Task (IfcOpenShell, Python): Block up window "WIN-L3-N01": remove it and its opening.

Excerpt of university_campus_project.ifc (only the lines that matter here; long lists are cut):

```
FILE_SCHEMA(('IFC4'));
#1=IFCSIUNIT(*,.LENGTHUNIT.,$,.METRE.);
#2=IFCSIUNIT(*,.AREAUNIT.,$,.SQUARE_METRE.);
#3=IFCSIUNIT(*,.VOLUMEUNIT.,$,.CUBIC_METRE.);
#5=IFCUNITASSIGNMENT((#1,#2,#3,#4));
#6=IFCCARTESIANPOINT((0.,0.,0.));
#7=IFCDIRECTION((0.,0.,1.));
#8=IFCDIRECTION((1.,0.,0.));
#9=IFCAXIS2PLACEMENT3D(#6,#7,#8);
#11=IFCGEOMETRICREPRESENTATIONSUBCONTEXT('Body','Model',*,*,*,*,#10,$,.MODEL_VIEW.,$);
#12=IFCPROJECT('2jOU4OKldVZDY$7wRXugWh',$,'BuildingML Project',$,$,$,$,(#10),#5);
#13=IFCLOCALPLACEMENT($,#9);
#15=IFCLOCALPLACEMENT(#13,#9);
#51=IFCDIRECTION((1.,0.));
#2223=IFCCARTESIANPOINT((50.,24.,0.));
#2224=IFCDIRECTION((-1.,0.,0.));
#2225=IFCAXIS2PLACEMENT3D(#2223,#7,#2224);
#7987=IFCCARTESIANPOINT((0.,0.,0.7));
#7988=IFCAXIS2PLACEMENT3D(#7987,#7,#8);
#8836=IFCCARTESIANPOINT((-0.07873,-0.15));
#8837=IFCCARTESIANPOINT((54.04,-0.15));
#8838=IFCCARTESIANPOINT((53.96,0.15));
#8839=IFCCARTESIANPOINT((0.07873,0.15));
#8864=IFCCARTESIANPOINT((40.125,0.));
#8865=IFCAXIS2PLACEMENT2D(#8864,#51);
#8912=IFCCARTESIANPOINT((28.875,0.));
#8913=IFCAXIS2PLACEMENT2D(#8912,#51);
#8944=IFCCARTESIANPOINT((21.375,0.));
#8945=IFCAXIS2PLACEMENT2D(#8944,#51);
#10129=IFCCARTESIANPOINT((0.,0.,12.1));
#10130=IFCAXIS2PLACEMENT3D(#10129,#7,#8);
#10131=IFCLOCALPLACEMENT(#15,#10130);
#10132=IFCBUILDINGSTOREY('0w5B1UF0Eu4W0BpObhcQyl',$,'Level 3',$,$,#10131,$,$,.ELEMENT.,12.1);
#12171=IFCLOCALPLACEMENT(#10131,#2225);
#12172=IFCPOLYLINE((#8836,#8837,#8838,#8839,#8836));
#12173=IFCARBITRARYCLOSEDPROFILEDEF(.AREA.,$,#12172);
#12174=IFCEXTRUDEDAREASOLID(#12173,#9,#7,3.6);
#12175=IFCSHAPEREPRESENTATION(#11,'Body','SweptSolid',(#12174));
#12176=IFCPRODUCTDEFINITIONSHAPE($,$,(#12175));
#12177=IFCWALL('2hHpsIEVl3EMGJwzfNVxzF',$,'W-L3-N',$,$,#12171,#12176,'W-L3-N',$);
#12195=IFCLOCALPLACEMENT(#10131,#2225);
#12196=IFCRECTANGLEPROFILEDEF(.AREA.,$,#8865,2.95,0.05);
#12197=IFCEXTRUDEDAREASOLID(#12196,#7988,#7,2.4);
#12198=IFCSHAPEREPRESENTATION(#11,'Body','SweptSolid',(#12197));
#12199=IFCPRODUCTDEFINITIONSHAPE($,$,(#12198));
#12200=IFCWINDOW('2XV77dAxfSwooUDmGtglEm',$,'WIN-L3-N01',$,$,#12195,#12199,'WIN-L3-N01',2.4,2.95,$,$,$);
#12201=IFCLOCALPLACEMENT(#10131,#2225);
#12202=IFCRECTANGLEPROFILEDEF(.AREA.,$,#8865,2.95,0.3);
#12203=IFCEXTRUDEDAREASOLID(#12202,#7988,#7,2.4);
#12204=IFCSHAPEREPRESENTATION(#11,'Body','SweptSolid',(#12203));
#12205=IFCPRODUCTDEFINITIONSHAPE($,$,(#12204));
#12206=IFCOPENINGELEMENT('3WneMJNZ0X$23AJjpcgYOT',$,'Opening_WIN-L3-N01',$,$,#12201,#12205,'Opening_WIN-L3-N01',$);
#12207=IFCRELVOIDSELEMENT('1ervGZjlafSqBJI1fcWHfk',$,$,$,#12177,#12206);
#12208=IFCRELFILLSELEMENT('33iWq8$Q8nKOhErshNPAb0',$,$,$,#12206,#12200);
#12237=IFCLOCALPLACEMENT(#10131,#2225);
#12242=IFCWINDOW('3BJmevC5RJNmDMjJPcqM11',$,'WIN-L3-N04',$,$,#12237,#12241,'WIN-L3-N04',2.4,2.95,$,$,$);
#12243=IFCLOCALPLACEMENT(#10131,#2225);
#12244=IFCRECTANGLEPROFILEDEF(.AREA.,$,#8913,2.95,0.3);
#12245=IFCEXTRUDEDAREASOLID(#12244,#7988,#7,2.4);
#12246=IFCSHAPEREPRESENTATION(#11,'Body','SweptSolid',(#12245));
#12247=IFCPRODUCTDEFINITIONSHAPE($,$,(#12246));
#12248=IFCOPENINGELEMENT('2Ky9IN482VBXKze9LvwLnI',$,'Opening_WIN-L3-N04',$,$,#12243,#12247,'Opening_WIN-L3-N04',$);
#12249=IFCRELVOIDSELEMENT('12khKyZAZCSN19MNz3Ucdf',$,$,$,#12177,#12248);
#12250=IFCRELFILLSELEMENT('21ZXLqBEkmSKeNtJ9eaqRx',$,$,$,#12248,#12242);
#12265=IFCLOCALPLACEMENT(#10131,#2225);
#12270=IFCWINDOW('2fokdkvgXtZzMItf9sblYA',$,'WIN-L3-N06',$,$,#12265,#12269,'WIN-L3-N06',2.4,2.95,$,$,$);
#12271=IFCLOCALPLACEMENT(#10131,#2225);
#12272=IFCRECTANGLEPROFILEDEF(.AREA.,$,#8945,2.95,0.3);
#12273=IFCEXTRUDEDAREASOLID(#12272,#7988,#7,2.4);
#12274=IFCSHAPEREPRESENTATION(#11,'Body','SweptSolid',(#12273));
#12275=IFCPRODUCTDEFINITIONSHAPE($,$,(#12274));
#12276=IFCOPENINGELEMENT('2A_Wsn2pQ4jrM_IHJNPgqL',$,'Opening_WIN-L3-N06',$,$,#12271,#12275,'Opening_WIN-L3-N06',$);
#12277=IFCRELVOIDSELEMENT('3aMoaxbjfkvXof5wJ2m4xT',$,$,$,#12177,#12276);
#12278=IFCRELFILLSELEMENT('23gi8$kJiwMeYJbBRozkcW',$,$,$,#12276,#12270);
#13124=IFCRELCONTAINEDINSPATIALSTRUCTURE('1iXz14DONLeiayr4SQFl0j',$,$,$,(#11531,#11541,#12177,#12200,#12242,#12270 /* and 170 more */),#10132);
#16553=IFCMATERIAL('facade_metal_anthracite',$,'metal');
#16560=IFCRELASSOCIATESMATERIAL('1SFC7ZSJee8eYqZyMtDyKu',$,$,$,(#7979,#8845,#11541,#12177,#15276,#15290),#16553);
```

```python
import ifcopenshell
import ifcopenshell.api.feature
import ifcopenshell.api.root
import ifcopenshell.geom
import ifcopenshell.util.shape

model = ifcopenshell.open("university_campus_project.ifc")
settings = ifcopenshell.geom.settings()


def volume(element):
    """Net volume in cubic metres, openings subtracted."""
    shape = ifcopenshell.geom.create_shape(settings, element)
    return ifcopenshell.util.shape.get_volume(shape.geometry)


window = model.by_guid("2XV77dAxfSwooUDmGtglEm")
opening = window.FillsVoids[0].RelatingOpeningElement
wall = opening.VoidsElements[0].RelatingBuildingElement
before = volume(wall)

ifcopenshell.api.root.remove_product(model, product=window)
ifcopenshell.api.feature.remove_feature(model, feature=opening)

after = volume(wall)

print(f"wall volume {before:.3f} -> {after:.3f} m3")

model.write("university_campus_project_rev.ifc")
```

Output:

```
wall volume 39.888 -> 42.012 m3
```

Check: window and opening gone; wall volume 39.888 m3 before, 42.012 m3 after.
